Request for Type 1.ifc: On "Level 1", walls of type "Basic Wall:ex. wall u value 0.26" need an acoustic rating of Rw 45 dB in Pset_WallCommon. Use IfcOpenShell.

First a look at what the model holds.

```python
import ifcopenshell
import ifcopenshell.util.element

model = ifcopenshell.open("Type 1.ifc")
print(model.schema)
storey = next(s for s in model.by_type("IfcBuildingStorey") if s.Name == "Level 1")
walls = [e for e in ifcopenshell.util.element.get_decomposition(storey) if e.is_a("IfcWall")]
seen = {}
for e in walls:
    element_type = ifcopenshell.util.element.get_type(e)
    key = (element_type.Name if element_type != e and element_type else None, ifcopenshell.util.element.get_pset(e, "Pset_WallCommon", "AcousticRating"))
    seen[key] = seen.get(key, 0) + 1
for (name, value), count in sorted(seen.items(), key=str):
    print(count, "x", name, "|", value)
```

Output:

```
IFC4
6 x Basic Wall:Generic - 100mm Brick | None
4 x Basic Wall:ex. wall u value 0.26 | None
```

```python
import ifcopenshell
import ifcopenshell.api.pset
import ifcopenshell.util.element

model = ifcopenshell.open("Type 1.ifc")

storey = next(s for s in model.by_type("IfcBuildingStorey") if s.Name == "Level 1")
walls = [e for e in ifcopenshell.util.element.get_decomposition(storey) if e.is_a("IfcWall")]

count = 0
for e in walls:
    element_type = ifcopenshell.util.element.get_type(e)
    if element_type in (None, e) or element_type.Name != "Basic Wall:ex. wall u value 0.26":
        continue
    # add_pset returns the element's existing set when there is one.
    pset = ifcopenshell.api.pset.add_pset(model, product=e, name="Pset_WallCommon")
    ifcopenshell.api.pset.edit_pset(model, pset=pset, properties={"AcousticRating": "Rw 45 dB"})
    count += 1

print(count, "walls updated")

model.write("Type 1_edited.ifc")
```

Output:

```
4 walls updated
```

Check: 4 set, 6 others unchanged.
